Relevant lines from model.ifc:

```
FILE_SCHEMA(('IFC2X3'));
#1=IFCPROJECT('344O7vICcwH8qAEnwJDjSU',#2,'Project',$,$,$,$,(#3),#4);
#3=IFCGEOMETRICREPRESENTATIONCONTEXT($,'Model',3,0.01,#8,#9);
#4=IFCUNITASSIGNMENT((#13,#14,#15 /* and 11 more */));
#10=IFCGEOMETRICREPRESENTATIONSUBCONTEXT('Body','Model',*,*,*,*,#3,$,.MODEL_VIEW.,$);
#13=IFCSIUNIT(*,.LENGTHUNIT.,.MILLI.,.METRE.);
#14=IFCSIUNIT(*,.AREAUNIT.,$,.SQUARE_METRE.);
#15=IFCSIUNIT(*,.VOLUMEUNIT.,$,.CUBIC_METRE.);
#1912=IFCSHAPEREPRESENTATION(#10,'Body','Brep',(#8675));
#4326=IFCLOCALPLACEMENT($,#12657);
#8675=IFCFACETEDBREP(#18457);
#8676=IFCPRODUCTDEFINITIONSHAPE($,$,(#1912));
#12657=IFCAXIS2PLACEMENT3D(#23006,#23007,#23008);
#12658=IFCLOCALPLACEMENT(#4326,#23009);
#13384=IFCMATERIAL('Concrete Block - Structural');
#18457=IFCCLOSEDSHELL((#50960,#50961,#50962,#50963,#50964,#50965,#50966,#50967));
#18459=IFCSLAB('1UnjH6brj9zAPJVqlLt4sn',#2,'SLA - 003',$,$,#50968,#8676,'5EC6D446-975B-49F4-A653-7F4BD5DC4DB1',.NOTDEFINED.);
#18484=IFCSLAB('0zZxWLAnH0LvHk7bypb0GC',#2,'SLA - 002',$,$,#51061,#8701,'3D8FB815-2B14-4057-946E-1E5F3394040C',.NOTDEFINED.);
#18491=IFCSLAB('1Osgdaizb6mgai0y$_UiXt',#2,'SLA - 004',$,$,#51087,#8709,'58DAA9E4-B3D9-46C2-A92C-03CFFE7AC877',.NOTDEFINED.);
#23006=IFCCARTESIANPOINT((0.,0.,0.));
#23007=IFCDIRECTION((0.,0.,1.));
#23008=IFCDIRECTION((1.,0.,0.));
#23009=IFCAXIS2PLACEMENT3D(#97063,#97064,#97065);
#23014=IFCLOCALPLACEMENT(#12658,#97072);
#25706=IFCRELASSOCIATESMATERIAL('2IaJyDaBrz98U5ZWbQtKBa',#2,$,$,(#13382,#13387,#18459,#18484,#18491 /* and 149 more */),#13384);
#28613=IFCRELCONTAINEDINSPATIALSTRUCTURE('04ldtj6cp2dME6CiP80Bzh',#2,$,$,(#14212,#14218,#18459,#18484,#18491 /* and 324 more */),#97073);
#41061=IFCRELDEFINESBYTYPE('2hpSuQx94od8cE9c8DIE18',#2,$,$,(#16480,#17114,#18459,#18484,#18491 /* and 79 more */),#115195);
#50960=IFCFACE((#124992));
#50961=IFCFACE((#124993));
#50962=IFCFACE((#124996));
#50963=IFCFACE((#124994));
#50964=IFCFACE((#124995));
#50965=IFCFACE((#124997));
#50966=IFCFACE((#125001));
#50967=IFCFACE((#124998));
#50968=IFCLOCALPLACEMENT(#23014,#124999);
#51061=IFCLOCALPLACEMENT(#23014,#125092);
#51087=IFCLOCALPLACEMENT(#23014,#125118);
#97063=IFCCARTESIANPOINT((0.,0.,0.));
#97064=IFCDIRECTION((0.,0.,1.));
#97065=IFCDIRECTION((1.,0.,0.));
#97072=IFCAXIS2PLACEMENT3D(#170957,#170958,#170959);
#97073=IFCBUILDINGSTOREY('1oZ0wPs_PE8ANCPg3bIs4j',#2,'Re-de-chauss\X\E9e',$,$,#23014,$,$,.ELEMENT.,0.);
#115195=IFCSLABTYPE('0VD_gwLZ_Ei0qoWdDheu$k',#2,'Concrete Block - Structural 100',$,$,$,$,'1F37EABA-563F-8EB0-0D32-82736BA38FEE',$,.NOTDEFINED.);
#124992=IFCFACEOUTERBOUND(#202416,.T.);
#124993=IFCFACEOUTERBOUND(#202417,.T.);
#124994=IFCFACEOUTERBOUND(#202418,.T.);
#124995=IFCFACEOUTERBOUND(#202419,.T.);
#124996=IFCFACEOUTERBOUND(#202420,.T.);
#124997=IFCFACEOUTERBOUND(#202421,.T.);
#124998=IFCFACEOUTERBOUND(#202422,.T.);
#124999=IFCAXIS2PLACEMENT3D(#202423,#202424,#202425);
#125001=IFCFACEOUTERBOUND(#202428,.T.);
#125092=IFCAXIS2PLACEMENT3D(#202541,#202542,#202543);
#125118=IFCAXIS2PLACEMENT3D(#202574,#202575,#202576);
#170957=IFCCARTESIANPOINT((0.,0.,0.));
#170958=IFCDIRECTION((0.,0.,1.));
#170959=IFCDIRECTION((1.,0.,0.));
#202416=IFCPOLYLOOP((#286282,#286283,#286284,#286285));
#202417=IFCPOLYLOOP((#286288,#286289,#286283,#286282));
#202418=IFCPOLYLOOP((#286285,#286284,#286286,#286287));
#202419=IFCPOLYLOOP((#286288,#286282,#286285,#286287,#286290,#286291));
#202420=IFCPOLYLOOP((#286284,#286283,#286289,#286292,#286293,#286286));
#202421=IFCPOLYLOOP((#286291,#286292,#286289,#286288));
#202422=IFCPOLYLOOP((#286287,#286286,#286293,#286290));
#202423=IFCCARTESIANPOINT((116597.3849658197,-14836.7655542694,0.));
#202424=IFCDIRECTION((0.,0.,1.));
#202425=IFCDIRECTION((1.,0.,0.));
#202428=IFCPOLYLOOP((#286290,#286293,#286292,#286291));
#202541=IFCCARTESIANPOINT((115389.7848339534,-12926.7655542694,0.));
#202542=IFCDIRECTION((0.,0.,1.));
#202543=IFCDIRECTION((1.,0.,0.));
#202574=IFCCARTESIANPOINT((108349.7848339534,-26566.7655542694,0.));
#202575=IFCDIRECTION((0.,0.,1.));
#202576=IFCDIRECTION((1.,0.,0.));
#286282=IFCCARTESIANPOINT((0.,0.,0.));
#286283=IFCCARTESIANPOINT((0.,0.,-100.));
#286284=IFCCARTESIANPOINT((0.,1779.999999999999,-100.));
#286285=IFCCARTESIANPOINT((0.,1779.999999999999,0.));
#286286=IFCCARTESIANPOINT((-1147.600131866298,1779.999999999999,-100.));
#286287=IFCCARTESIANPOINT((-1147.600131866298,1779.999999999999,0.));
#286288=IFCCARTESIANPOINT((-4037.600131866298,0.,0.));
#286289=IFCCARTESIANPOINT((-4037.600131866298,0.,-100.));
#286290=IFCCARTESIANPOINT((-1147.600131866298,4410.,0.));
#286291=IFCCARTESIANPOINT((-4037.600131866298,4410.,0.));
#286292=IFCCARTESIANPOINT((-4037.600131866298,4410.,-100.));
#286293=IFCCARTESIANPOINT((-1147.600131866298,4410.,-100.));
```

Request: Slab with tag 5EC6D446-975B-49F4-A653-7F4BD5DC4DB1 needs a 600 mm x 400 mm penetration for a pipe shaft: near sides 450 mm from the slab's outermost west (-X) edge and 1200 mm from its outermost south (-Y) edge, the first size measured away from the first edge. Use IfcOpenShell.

```python
import numpy as np
import ifcopenshell
import ifcopenshell.api.feature
import ifcopenshell.api.geometry
import ifcopenshell.api.root
import ifcopenshell.geom
import ifcopenshell.util.placement
import ifcopenshell.util.representation
import ifcopenshell.util.shape
import ifcopenshell.util.unit

model = ifcopenshell.open("model.ifc")
unit_scale = ifcopenshell.util.unit.calculate_unit_scale(model)
settings = ifcopenshell.geom.settings()


def volume(element):
    """Net volume in cubic metres, openings subtracted."""
    shape = ifcopenshell.geom.create_shape(settings, element)
    return ifcopenshell.util.shape.get_volume(shape.geometry)


slab = model.by_id(18459)
before = volume(slab)

# Extent in the slab's own axes, in metres. The edges named are its -X and -Y sides.
slab_shape = ifcopenshell.geom.create_shape(settings, slab)
vertices = ifcopenshell.util.shape.get_vertices(slab_shape.geometry)
x_min, y_min, bottom = vertices.min(axis=0)
top = vertices[:, 2].max()

opening = ifcopenshell.api.root.create_entity(model, ifc_class="IfcOpeningElement", name="Pipe shaft opening")
context = ifcopenshell.util.representation.get_context(model, "Model", "Body", "MODEL_VIEW")
width, depth = 0.6, 0.4
outline = [(0.0, 0.0), (width, 0.0), (width, depth), (0.0, depth), (0.0, 0.0)]
# Overshoot both faces by 50 mm so the cut is clean.
shape = ifcopenshell.api.geometry.add_slab_representation(
    model, context=context, depth=top - bottom + 0.1, polyline=outline
)
ifcopenshell.api.geometry.assign_representation(model, product=opening, representation=shape)

matrix = ifcopenshell.util.placement.get_local_placement(slab.ObjectPlacement)
matrix[:, 3] = matrix @ np.append(np.array([x_min + 0.45, y_min + 1.2, bottom - 0.05]) / unit_scale, 1.0)
ifcopenshell.api.geometry.edit_object_placement(model, product=opening, matrix=matrix, is_si=False)
ifcopenshell.api.feature.add_feature(model, feature=opening, element=slab)

after = volume(slab)

print(f"slab volume {before:.3f} -> {after:.3f} m3")

model.write("model-out.ifc")
```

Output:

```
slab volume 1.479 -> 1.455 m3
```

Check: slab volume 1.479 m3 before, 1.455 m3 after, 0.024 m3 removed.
